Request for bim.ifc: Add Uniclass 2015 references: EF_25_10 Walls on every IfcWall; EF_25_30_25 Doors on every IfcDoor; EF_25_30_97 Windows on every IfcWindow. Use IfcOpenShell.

First a look at what the model holds.

```python
import ifcopenshell

model = ifcopenshell.open("bim.ifc")
print(model.schema)
print("classifications:", [c.Name for c in model.by_type("IfcClassification")])
for ifc_class in ("IfcDoor", "IfcRoof", "IfcStair", "IfcWall", "IfcWindow"):
    print(ifc_class, len(model.by_type(ifc_class)))
```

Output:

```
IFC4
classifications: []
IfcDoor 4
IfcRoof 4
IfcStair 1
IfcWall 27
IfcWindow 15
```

```python
import ifcopenshell
import ifcopenshell.api.classification

model = ifcopenshell.open("bim.ifc")

system = ifcopenshell.api.classification.add_classification(model, classification="Uniclass 2015")

codes = {
    "IfcWall": ("EF_25_10", "Walls"),
    "IfcDoor": ("EF_25_30_25", "Doors"),
    "IfcWindow": ("EF_25_30_97", "Windows"),
}
for ifc_class, (code, name) in codes.items():
    products = model.by_type(ifc_class)
    ifcopenshell.api.classification.add_reference(
        model, products=products, classification=system, identification=code, name=name
    )
    print(code, len(products))

model.write("bim_edited.ifc")
```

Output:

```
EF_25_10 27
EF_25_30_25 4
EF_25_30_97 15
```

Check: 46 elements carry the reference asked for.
